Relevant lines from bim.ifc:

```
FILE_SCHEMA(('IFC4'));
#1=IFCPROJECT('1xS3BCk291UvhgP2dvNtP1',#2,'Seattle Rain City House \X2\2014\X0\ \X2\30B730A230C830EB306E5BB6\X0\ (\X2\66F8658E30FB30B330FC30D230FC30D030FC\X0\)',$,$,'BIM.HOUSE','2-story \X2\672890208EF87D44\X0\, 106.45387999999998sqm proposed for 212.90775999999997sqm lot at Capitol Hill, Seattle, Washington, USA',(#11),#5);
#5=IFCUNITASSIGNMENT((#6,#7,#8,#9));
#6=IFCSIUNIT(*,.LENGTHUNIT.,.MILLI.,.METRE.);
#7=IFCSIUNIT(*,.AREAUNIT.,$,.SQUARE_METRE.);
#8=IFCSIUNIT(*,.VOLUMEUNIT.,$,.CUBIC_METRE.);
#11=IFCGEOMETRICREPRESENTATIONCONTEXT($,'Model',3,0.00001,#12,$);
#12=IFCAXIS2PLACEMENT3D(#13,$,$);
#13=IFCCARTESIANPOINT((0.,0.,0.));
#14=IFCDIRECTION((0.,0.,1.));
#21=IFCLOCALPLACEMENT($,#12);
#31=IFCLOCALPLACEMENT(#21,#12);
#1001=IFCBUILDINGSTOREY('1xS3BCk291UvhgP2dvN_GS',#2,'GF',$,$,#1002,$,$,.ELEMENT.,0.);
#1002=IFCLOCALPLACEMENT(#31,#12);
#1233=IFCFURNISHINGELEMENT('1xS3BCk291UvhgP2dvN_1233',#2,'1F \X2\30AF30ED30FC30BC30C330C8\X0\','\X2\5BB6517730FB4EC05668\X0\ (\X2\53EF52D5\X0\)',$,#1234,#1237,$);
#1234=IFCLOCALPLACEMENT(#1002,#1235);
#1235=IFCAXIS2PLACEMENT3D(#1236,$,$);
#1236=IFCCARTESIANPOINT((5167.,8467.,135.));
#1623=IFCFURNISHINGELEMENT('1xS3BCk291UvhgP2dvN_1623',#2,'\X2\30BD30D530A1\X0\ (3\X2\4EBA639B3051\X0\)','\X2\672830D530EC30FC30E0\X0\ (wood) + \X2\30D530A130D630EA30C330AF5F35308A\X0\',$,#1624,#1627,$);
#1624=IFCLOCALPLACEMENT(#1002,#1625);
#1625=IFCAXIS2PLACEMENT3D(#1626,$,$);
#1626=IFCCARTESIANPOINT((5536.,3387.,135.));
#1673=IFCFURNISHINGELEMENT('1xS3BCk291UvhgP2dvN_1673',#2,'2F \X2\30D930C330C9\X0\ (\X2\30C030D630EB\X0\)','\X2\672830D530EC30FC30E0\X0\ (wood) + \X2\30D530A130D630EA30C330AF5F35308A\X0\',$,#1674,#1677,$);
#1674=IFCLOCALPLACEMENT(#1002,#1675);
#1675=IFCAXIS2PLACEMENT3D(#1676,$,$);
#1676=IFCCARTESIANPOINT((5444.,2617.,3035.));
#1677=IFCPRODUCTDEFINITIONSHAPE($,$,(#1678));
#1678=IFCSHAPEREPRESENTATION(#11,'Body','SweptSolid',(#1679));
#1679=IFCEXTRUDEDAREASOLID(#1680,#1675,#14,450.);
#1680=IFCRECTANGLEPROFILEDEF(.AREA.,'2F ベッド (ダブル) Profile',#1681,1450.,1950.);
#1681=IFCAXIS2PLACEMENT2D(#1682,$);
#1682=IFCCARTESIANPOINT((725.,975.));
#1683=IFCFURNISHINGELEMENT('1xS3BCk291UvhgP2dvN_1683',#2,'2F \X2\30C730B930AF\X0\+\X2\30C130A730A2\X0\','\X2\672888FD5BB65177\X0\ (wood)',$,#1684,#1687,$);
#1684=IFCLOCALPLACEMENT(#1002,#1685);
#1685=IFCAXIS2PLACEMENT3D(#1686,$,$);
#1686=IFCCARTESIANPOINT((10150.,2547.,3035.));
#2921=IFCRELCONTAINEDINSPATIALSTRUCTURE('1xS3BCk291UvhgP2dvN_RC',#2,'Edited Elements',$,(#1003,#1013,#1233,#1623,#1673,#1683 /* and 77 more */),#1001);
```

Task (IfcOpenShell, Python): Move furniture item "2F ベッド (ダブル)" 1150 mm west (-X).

```python
import ifcopenshell
import ifcopenshell.api.geometry
import ifcopenshell.util.placement
import ifcopenshell.util.unit

model = ifcopenshell.open("bim.ifc")
unit_scale = ifcopenshell.util.unit.calculate_unit_scale(model)

item = model.by_id(1673)
matrix = ifcopenshell.util.placement.get_local_placement(item.ObjectPlacement)
matrix[0, 3] -= 1.15 / unit_scale
ifcopenshell.api.geometry.edit_object_placement(model, product=item, matrix=matrix, is_si=False)

print(ifcopenshell.util.placement.get_local_placement(item.ObjectPlacement).round(3) + 0.0)

model.write("bim_rev.ifc")
```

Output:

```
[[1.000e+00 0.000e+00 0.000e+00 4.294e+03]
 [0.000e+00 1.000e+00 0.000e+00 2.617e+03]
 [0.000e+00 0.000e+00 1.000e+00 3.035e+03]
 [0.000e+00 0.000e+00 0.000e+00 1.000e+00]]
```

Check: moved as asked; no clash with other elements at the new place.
